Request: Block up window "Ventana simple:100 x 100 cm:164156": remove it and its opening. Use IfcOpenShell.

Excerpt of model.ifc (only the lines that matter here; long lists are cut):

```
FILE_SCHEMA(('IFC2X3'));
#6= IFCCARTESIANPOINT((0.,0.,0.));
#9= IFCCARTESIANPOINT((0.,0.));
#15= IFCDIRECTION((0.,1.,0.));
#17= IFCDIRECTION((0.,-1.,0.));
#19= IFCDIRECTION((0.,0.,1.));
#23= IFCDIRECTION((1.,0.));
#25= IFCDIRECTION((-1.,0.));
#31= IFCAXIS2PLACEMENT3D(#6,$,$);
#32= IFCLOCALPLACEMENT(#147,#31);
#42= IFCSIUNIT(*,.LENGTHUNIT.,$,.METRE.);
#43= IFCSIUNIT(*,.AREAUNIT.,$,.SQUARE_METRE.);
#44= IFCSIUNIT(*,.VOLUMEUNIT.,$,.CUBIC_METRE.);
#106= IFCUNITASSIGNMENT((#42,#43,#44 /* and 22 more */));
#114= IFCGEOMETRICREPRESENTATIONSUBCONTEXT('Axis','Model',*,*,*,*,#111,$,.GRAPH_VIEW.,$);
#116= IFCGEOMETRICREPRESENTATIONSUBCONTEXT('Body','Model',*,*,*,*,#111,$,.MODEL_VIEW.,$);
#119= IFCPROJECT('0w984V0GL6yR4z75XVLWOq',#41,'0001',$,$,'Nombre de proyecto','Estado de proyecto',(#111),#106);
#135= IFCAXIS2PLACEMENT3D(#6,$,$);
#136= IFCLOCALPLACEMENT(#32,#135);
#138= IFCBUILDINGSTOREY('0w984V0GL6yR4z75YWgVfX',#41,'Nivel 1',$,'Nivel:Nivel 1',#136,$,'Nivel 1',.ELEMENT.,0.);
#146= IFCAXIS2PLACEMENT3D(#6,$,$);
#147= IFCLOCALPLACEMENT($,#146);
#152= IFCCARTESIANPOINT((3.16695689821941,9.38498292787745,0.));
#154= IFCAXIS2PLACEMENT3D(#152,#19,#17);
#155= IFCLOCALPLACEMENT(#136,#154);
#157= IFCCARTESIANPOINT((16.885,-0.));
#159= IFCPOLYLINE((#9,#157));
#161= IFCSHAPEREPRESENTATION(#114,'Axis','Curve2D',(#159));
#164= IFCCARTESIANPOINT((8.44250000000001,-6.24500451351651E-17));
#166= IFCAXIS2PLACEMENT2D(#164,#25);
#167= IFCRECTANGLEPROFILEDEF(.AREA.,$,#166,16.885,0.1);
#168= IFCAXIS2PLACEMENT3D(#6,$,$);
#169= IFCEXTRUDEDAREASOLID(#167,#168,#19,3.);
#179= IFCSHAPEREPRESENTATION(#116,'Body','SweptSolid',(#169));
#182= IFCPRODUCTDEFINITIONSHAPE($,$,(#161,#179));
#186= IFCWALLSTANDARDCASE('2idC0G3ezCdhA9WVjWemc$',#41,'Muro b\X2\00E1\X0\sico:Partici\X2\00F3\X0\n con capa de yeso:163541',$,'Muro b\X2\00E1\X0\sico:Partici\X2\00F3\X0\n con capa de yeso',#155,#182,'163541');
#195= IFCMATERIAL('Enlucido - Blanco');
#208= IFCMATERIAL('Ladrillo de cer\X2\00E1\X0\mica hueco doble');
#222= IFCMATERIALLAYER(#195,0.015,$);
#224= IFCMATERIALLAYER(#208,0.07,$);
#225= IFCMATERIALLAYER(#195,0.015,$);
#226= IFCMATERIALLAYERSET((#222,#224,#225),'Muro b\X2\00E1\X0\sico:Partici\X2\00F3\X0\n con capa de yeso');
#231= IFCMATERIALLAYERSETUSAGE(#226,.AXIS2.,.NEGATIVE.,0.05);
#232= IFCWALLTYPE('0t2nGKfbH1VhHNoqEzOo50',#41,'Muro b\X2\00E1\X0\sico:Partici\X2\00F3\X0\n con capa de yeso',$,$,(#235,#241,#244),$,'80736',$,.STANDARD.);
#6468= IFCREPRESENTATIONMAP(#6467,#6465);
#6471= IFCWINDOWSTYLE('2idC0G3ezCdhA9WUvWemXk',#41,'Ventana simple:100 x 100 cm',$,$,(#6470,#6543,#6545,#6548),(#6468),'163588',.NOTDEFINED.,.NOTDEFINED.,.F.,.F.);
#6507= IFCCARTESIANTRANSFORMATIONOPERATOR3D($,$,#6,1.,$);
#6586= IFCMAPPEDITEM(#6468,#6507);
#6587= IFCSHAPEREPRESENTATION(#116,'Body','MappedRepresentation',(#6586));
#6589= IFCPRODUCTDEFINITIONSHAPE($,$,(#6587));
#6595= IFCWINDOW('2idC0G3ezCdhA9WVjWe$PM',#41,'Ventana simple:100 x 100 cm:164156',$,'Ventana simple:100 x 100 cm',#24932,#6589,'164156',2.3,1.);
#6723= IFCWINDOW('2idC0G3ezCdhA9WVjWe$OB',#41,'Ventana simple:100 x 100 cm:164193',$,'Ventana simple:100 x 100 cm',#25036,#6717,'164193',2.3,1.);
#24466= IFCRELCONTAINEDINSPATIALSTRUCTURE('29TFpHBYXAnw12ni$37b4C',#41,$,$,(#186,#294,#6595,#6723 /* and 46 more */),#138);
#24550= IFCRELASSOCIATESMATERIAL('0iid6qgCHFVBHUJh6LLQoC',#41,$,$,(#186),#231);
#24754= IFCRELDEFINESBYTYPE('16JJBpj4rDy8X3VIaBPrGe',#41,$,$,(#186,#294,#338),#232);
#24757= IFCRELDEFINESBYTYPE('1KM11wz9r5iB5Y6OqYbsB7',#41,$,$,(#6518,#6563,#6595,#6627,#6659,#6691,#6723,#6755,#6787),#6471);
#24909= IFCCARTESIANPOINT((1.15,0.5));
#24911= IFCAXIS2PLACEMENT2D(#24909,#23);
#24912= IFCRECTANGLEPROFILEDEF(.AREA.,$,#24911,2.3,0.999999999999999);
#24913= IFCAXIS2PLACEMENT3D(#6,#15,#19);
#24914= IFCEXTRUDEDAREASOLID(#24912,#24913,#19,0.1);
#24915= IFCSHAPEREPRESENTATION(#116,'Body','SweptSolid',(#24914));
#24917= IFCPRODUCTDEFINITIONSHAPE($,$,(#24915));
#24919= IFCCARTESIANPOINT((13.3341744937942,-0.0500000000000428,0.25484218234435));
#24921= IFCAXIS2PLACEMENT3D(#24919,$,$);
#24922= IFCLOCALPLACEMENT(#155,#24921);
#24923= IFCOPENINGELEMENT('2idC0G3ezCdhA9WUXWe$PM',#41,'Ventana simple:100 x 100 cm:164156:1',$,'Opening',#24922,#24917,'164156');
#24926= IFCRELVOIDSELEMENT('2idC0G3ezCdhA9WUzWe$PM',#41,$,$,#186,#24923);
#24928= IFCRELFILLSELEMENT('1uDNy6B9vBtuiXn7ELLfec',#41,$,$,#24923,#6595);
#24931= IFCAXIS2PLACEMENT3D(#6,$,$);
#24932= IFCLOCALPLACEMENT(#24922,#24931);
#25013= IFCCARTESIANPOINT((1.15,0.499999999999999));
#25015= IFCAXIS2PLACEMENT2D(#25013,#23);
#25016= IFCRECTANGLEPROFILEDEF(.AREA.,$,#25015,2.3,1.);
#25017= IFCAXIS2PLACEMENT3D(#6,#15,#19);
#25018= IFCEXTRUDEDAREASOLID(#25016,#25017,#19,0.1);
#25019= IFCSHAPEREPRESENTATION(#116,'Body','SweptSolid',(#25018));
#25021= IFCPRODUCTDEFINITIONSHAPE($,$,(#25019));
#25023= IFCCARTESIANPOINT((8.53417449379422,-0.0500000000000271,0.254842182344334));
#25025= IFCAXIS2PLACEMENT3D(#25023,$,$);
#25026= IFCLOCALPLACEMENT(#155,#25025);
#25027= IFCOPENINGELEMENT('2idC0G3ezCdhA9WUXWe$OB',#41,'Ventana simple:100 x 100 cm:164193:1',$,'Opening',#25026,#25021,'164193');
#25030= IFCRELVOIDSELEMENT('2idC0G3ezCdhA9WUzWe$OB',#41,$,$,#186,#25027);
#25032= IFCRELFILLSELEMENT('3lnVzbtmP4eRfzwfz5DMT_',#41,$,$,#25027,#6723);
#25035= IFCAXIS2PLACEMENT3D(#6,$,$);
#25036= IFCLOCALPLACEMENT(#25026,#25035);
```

```python
import ifcopenshell
import ifcopenshell.api.feature
import ifcopenshell.api.root
import ifcopenshell.geom
import ifcopenshell.util.shape

model = ifcopenshell.open("model.ifc")
settings = ifcopenshell.geom.settings()


def volume(element):
    """Net volume in cubic metres, openings subtracted."""
    shape = ifcopenshell.geom.create_shape(settings, element)
    return ifcopenshell.util.shape.get_volume(shape.geometry)


window = model.by_guid("2idC0G3ezCdhA9WVjWe$PM")
opening = window.FillsVoids[0].RelatingOpeningElement
wall = opening.VoidsElements[0].RelatingBuildingElement
before = volume(wall)

ifcopenshell.api.root.remove_product(model, product=window)
ifcopenshell.api.feature.remove_feature(model, feature=opening)

after = volume(wall)

print(f"wall volume {before:.3f} -> {after:.3f} m3")

model.write("model-out.ifc")
```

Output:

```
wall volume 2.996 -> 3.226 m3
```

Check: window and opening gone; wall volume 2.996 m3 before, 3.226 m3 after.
